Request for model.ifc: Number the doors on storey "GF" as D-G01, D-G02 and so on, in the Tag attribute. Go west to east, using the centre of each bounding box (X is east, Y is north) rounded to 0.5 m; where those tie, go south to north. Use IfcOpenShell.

First a look at what the model holds.

```python
import ifcopenshell
import ifcopenshell.util.element
import ifcopenshell.util.placement

model = ifcopenshell.open("model.ifc")
print(model.schema)
storey = next(s for s in model.by_type("IfcBuildingStorey") if s.Name == "GF")
doors = [e for e in ifcopenshell.util.element.get_decomposition(storey) if e.is_a("IfcDoor")]
for e in sorted(doors, key=lambda e: e.id()):
    origin = ifcopenshell.util.placement.get_local_placement(e.ObjectPlacement)[:3, 3]
    print(e.id(), e.Tag, e.Name, origin.round(2) + 0.0, sep=" | ")
```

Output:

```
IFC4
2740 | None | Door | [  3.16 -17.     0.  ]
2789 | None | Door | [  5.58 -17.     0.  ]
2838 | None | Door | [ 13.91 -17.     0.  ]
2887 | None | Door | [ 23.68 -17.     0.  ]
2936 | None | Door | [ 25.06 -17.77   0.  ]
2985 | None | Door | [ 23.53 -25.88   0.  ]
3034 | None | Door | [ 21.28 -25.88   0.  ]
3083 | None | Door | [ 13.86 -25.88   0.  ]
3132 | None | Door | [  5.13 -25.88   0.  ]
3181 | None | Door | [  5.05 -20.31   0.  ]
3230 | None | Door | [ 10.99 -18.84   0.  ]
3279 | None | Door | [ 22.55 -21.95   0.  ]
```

```python
import ifcopenshell
import ifcopenshell.geom
import ifcopenshell.util.element
import ifcopenshell.util.shape

model = ifcopenshell.open("model.ifc")
settings = ifcopenshell.geom.settings()
settings.set("use-world-coords", True)


def centre(element):
    shape = ifcopenshell.geom.create_shape(settings, element)
    return ifcopenshell.util.shape.get_bbox_centroid(shape.geometry)


storey = next(s for s in model.by_type("IfcBuildingStorey") if s.Name == "GF")
doors = [e for e in ifcopenshell.util.element.get_decomposition(storey) if e.is_a("IfcDoor")]

# Insertion points can sit at a corner or the storey origin, so sort by the geometry (in metres).
centres = {e: centre(e) for e in doors}
doors.sort(key=lambda e: (round(centres[e][0] / 0.5), centres[e][1]))

for i, e in enumerate(doors, start=1):
    number = f"D-G{i:02d}"
    e.Tag = number
    print(e.id(), number)

model.write("model_updated.ifc")
```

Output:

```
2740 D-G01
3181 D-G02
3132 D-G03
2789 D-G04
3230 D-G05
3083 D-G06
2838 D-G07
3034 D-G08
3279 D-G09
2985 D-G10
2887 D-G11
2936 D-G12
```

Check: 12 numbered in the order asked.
